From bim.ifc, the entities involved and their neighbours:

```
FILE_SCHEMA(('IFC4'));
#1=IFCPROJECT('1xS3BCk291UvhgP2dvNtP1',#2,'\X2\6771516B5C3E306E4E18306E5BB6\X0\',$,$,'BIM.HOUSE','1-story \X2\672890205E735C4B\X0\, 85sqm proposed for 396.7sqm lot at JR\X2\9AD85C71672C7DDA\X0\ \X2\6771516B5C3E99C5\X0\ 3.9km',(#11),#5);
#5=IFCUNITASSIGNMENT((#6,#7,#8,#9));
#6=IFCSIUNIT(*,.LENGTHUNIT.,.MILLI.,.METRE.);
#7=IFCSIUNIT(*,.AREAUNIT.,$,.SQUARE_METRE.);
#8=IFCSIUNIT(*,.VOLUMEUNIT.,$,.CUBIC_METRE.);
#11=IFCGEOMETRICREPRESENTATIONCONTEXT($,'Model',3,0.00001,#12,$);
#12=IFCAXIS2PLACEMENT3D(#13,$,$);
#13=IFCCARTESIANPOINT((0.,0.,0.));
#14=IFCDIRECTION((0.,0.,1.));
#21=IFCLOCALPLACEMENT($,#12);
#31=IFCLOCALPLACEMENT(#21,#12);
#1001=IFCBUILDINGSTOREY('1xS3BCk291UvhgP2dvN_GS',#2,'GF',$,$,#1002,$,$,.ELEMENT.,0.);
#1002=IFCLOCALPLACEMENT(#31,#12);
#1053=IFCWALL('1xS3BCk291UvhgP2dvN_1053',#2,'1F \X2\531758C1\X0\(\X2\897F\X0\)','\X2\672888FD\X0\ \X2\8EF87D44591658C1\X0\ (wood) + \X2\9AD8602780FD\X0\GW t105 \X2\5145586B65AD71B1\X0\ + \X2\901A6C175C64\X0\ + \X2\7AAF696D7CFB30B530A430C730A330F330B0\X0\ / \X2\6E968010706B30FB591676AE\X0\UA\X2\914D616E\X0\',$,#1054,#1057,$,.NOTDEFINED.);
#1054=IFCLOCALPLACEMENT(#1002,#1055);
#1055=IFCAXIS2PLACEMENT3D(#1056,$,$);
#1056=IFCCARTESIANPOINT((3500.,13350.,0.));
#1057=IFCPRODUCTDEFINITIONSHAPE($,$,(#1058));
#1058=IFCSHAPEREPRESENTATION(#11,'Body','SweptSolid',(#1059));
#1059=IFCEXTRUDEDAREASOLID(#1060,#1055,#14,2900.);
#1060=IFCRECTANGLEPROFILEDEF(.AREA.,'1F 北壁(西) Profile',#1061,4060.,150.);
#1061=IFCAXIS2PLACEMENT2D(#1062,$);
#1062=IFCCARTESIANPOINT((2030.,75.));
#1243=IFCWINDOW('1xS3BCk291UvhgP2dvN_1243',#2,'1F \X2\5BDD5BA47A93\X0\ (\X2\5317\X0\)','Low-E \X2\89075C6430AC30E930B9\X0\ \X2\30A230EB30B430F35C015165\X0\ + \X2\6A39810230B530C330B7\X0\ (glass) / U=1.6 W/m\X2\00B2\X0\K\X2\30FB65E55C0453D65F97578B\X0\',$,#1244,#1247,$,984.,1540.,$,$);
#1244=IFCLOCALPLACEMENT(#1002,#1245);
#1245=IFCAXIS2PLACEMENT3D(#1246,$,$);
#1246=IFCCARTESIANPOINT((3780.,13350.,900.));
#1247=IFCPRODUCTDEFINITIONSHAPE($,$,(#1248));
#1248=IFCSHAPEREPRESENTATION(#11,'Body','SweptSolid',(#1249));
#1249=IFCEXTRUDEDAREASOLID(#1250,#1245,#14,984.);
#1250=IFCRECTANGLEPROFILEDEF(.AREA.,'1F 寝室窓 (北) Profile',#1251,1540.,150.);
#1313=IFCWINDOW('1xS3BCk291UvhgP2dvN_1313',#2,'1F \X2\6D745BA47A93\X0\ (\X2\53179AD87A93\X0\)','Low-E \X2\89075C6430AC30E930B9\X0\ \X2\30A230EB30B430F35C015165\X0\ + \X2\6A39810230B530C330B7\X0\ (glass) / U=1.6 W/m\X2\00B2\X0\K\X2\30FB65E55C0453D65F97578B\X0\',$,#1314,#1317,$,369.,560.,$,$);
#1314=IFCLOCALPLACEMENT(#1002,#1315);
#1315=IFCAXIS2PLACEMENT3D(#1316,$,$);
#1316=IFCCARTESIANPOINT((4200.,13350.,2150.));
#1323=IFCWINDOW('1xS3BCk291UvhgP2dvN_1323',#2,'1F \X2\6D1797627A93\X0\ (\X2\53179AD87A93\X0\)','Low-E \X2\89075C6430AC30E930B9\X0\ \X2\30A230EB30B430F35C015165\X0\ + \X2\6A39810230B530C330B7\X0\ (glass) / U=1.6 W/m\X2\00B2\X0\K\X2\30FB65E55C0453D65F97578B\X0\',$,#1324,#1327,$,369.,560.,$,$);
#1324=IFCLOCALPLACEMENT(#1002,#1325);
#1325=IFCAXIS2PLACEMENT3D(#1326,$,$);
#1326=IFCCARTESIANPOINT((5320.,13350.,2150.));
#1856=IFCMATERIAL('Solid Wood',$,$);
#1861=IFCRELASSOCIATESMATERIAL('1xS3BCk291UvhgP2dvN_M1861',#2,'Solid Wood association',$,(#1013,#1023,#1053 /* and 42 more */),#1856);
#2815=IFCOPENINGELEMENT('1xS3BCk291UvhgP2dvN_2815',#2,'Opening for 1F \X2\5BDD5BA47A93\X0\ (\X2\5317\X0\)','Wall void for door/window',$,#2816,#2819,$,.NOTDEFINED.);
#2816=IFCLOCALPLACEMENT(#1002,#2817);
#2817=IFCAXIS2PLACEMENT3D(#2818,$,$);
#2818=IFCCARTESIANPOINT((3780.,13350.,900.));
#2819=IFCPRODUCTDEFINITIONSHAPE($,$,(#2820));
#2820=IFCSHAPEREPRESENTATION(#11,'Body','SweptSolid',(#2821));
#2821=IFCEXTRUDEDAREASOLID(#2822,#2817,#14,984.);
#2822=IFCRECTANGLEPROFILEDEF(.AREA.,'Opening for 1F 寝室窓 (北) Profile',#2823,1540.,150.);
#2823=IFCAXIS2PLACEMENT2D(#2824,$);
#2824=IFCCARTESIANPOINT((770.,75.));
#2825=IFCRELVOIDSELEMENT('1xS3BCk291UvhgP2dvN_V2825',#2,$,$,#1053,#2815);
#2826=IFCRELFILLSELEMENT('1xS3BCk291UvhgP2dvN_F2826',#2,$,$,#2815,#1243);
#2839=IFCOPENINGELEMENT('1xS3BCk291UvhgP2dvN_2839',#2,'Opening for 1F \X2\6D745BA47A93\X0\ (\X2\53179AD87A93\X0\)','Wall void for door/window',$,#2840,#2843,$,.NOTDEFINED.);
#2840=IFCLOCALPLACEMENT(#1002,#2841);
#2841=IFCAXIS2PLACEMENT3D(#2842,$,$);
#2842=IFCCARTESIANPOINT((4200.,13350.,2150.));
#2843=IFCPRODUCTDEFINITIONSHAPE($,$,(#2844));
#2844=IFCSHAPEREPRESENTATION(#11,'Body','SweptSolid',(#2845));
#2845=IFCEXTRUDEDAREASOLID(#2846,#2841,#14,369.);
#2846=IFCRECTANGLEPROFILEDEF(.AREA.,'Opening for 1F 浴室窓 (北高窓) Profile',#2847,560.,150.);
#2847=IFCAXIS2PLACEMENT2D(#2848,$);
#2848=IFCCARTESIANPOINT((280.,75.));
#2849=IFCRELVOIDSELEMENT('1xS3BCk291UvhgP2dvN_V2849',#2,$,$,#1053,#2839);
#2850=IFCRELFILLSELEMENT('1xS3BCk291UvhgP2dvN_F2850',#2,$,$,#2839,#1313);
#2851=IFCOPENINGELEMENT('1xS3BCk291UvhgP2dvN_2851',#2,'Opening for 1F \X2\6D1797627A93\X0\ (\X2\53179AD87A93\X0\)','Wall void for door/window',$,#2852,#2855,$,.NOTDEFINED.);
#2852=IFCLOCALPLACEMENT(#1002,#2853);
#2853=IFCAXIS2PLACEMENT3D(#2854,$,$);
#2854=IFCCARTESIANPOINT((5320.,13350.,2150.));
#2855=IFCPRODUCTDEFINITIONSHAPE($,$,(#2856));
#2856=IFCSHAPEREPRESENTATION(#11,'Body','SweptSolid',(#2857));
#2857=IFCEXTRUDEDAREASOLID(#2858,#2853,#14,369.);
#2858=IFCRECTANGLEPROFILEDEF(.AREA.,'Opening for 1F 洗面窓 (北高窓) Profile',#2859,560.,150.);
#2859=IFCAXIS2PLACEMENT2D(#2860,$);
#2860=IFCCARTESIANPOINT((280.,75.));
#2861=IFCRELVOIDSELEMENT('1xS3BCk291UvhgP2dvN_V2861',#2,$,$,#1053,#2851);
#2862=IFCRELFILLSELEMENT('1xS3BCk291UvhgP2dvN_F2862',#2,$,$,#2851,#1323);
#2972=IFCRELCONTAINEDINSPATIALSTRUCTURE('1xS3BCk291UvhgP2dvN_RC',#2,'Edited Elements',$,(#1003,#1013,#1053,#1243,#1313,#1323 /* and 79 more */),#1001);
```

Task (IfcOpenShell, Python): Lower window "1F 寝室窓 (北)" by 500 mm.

```python
import numpy as np
import ifcopenshell
import ifcopenshell.api.geometry
import ifcopenshell.util.placement
import ifcopenshell.util.unit

model = ifcopenshell.open("bim.ifc")
unit_scale = ifcopenshell.util.unit.calculate_unit_scale(model)

window = model.by_id(1243)
opening = window.FillsVoids[0].RelatingOpeningElement
dz = -500.0

shift = np.array([0.0, 0.0, dz])
# The window is not placed relative to its opening, so move both.
for product in (opening, window):
    matrix = ifcopenshell.util.placement.get_local_placement(product.ObjectPlacement)
    matrix[:3, 3] += shift
    ifcopenshell.api.geometry.edit_object_placement(model, product=product, matrix=matrix, is_si=False)

print(f"moved by {dz * unit_scale:+.3f} m")

model.write("bim_rev.ifc")
```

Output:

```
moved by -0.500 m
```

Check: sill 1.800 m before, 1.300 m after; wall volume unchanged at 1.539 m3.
